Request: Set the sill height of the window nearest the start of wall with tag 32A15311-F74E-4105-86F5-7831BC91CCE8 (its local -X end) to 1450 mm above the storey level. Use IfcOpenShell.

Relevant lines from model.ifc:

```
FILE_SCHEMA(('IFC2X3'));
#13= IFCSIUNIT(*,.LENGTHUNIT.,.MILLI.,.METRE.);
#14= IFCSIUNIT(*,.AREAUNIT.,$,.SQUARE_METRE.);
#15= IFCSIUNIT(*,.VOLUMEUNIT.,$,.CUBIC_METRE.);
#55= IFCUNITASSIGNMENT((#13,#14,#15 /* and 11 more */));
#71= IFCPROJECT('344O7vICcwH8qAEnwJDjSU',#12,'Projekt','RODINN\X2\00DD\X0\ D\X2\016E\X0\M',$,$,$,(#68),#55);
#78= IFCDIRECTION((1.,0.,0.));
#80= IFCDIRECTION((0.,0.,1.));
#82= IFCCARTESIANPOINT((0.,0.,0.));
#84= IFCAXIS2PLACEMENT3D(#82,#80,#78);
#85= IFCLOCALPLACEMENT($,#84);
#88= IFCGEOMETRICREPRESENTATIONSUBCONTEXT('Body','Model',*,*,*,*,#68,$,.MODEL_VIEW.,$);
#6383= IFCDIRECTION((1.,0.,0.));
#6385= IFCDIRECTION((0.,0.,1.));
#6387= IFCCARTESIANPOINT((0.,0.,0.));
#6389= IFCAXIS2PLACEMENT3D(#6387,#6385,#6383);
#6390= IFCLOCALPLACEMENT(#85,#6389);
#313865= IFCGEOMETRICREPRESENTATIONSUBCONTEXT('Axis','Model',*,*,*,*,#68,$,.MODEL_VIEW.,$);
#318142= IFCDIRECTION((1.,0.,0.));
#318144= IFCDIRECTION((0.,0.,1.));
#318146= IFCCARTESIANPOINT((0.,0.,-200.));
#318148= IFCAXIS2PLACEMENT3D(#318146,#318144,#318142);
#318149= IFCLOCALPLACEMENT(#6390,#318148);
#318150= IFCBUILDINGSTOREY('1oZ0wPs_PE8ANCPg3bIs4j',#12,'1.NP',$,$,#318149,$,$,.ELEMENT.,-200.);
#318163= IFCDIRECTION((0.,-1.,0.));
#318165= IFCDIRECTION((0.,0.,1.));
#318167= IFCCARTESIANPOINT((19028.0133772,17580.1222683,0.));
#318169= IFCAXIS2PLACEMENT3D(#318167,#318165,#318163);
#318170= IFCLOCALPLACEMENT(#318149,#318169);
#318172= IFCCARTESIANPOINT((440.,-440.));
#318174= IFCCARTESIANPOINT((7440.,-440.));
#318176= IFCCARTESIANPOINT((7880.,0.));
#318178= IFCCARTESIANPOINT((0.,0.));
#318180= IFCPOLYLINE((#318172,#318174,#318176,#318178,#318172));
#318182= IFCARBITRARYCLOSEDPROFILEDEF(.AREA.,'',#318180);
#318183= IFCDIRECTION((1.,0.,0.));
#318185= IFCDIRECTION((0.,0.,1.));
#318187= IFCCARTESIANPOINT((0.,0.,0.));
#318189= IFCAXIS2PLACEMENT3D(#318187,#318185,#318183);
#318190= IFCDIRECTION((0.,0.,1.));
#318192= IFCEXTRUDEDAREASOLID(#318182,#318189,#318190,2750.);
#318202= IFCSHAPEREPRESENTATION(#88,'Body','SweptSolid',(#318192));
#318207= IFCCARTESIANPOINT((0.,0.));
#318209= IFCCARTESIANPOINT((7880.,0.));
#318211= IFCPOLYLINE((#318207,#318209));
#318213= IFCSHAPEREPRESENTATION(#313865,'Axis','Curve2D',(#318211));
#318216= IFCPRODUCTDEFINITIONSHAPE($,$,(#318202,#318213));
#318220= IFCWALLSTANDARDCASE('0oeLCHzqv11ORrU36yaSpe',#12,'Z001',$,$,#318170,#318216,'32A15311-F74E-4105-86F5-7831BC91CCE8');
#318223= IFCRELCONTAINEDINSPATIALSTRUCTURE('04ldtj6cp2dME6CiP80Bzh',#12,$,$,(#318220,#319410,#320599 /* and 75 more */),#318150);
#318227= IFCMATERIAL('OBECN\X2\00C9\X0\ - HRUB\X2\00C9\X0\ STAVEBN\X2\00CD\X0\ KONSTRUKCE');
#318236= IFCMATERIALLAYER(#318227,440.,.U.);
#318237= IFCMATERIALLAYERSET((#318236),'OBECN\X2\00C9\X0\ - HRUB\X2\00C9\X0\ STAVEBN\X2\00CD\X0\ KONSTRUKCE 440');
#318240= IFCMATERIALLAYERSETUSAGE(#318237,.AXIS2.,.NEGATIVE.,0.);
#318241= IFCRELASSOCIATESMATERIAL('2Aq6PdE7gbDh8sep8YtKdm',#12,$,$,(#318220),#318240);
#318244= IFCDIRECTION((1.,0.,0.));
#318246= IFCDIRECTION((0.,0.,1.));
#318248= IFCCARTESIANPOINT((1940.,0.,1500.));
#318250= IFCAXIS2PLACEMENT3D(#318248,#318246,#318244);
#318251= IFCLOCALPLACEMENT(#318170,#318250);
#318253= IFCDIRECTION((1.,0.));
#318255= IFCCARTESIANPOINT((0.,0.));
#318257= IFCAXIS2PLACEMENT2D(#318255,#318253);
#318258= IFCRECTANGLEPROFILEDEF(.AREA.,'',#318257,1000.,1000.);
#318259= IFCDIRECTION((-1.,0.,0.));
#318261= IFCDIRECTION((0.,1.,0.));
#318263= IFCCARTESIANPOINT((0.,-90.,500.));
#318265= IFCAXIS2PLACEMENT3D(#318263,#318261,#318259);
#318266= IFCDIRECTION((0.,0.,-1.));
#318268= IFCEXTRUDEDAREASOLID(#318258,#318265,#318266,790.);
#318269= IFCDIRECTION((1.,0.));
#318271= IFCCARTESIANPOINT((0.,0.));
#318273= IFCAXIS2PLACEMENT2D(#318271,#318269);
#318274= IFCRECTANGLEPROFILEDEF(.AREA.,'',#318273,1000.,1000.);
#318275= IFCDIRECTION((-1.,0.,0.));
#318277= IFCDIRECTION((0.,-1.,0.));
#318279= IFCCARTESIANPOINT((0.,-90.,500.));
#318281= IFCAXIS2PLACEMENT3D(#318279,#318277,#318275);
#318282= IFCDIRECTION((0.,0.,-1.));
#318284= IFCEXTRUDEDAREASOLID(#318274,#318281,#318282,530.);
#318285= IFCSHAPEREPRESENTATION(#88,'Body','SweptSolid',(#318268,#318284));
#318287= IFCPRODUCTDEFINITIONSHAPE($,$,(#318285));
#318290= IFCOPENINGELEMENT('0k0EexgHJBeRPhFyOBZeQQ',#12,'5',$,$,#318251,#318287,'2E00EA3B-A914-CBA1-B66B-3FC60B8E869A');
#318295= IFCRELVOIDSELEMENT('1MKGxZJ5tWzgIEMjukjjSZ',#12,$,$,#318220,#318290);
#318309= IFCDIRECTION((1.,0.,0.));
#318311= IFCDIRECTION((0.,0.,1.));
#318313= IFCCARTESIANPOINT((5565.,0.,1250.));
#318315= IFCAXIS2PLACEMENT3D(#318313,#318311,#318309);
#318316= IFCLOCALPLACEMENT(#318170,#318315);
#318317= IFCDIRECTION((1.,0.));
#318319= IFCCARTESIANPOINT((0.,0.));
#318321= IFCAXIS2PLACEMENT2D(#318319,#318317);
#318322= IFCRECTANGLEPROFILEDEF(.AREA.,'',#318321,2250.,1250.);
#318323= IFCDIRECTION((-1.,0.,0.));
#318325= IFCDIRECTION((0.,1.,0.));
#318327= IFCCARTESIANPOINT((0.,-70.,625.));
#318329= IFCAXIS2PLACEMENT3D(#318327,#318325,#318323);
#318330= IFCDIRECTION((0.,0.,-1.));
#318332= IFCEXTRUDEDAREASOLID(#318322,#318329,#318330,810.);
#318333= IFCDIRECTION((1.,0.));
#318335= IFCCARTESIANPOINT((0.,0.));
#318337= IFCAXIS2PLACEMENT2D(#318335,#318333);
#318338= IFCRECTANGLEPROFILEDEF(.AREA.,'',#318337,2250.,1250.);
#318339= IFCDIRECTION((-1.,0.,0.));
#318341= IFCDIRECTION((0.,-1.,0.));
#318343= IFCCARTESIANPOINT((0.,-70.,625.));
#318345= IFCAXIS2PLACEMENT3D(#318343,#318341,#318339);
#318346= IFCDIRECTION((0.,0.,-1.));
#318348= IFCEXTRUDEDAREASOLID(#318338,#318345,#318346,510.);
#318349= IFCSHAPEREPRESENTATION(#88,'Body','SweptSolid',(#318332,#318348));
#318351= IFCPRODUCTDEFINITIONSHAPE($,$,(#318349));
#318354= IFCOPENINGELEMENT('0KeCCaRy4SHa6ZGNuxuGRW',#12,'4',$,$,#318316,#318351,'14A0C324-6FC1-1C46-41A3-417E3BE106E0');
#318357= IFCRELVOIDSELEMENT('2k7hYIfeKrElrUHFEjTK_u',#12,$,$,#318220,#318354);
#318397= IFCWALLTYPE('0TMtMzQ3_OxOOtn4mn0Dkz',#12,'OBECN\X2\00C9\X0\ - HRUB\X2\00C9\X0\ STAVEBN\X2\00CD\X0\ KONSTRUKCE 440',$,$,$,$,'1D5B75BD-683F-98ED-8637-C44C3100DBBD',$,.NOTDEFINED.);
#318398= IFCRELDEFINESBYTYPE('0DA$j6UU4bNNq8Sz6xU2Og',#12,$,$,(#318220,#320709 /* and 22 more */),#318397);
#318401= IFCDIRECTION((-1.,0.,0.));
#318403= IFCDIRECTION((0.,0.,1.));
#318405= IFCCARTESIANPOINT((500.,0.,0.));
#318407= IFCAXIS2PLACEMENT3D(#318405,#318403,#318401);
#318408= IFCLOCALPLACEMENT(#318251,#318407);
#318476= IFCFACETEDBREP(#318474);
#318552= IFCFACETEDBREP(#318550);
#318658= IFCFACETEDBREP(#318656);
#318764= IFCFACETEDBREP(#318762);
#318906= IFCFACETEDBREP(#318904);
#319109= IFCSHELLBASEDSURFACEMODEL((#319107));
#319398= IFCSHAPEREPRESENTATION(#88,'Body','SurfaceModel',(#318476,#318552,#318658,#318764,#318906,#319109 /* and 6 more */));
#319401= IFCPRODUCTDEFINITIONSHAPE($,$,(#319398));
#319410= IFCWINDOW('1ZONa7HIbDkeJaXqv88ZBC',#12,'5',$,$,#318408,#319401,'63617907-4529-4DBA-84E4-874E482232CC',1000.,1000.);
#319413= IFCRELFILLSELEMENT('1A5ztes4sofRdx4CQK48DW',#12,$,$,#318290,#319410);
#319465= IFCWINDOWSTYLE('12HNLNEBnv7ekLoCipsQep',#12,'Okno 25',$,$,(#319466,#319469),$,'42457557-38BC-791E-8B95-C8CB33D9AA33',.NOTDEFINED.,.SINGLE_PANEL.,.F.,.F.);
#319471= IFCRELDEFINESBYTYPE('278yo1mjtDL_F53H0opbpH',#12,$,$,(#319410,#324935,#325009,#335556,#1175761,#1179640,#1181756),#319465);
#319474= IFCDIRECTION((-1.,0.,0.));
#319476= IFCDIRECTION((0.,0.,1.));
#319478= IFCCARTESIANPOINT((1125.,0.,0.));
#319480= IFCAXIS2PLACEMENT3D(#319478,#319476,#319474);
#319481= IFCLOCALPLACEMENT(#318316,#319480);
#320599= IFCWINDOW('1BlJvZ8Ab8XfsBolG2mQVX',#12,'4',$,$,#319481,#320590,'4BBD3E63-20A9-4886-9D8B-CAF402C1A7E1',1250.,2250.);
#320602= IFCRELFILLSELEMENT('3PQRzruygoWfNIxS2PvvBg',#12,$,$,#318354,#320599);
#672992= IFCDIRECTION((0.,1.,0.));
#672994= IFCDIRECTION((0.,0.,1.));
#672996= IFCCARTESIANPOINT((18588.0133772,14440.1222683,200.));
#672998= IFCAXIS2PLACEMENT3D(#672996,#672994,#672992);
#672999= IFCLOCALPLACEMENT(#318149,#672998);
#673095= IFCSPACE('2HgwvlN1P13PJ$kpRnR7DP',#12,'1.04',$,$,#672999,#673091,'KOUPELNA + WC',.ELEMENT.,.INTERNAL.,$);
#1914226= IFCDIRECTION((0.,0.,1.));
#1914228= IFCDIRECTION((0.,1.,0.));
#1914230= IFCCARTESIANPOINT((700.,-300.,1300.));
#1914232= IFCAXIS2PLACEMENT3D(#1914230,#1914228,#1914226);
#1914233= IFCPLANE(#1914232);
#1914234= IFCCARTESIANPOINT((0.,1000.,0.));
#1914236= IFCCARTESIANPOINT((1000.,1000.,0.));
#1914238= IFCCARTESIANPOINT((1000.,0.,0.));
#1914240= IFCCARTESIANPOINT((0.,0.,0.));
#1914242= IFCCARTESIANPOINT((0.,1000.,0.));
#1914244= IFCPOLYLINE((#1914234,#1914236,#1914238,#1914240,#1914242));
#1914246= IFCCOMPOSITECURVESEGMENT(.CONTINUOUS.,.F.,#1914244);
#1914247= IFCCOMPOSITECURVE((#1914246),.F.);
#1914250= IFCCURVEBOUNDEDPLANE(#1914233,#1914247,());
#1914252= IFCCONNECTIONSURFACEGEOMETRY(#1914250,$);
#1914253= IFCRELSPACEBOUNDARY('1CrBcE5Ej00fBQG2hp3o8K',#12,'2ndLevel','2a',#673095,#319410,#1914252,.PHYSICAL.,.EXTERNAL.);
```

```python
import numpy as np
import ifcopenshell
import ifcopenshell.api.geometry
import ifcopenshell.geom
import ifcopenshell.util.element
import ifcopenshell.util.placement
import ifcopenshell.util.shape
import ifcopenshell.util.unit

model = ifcopenshell.open("model.ifc")
unit_scale = ifcopenshell.util.unit.calculate_unit_scale(model)

window = model.by_id(319410)
opening = window.FillsVoids[0].RelatingOpeningElement
storey = ifcopenshell.util.element.get_container(window, ifc_class="IfcBuildingStorey")
level = ifcopenshell.util.placement.get_local_placement(storey.ObjectPlacement)[2, 3]

# The opening's origin need not be at the sill, so measure its lowest point.
shape = ifcopenshell.geom.create_shape(ifcopenshell.geom.settings(), opening)
bottom = ifcopenshell.util.shape.get_shape_bottom_elevation(shape, shape.geometry) / unit_scale
dz = level + 1.45 / unit_scale - bottom

shift = np.array([0.0, 0.0, dz])
# The window is placed relative to its opening, so it follows when the opening moves.
matrix = ifcopenshell.util.placement.get_local_placement(opening.ObjectPlacement)
matrix[:3, 3] += shift
ifcopenshell.api.geometry.edit_object_placement(
    model, product=opening, matrix=matrix, is_si=False, should_transform_children=True
)

# Space boundary surfaces are stored in each space's coordinates; move them too.
for rel in window.ProvidesBoundaries:
    if not rel.ConnectionGeometry:
        continue
    surface = rel.ConnectionGeometry.SurfaceOnRelatingElement.BasisSurface
    space_matrix = ifcopenshell.util.placement.get_local_placement(rel.RelatingSpace.ObjectPlacement)
    point = np.array(surface.Position.Location.Coordinates) + space_matrix[:3, :3].T @ shift
    surface.Position = model.createIfcAxis2Placement3D(
        model.createIfcCartesianPoint(point.tolist()), surface.Position.Axis, surface.Position.RefDirection
    )

print(f"moved by {dz * unit_scale:+.3f} m")

model.write("model-out.ifc")
```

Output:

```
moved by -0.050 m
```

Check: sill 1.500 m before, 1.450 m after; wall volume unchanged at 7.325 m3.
